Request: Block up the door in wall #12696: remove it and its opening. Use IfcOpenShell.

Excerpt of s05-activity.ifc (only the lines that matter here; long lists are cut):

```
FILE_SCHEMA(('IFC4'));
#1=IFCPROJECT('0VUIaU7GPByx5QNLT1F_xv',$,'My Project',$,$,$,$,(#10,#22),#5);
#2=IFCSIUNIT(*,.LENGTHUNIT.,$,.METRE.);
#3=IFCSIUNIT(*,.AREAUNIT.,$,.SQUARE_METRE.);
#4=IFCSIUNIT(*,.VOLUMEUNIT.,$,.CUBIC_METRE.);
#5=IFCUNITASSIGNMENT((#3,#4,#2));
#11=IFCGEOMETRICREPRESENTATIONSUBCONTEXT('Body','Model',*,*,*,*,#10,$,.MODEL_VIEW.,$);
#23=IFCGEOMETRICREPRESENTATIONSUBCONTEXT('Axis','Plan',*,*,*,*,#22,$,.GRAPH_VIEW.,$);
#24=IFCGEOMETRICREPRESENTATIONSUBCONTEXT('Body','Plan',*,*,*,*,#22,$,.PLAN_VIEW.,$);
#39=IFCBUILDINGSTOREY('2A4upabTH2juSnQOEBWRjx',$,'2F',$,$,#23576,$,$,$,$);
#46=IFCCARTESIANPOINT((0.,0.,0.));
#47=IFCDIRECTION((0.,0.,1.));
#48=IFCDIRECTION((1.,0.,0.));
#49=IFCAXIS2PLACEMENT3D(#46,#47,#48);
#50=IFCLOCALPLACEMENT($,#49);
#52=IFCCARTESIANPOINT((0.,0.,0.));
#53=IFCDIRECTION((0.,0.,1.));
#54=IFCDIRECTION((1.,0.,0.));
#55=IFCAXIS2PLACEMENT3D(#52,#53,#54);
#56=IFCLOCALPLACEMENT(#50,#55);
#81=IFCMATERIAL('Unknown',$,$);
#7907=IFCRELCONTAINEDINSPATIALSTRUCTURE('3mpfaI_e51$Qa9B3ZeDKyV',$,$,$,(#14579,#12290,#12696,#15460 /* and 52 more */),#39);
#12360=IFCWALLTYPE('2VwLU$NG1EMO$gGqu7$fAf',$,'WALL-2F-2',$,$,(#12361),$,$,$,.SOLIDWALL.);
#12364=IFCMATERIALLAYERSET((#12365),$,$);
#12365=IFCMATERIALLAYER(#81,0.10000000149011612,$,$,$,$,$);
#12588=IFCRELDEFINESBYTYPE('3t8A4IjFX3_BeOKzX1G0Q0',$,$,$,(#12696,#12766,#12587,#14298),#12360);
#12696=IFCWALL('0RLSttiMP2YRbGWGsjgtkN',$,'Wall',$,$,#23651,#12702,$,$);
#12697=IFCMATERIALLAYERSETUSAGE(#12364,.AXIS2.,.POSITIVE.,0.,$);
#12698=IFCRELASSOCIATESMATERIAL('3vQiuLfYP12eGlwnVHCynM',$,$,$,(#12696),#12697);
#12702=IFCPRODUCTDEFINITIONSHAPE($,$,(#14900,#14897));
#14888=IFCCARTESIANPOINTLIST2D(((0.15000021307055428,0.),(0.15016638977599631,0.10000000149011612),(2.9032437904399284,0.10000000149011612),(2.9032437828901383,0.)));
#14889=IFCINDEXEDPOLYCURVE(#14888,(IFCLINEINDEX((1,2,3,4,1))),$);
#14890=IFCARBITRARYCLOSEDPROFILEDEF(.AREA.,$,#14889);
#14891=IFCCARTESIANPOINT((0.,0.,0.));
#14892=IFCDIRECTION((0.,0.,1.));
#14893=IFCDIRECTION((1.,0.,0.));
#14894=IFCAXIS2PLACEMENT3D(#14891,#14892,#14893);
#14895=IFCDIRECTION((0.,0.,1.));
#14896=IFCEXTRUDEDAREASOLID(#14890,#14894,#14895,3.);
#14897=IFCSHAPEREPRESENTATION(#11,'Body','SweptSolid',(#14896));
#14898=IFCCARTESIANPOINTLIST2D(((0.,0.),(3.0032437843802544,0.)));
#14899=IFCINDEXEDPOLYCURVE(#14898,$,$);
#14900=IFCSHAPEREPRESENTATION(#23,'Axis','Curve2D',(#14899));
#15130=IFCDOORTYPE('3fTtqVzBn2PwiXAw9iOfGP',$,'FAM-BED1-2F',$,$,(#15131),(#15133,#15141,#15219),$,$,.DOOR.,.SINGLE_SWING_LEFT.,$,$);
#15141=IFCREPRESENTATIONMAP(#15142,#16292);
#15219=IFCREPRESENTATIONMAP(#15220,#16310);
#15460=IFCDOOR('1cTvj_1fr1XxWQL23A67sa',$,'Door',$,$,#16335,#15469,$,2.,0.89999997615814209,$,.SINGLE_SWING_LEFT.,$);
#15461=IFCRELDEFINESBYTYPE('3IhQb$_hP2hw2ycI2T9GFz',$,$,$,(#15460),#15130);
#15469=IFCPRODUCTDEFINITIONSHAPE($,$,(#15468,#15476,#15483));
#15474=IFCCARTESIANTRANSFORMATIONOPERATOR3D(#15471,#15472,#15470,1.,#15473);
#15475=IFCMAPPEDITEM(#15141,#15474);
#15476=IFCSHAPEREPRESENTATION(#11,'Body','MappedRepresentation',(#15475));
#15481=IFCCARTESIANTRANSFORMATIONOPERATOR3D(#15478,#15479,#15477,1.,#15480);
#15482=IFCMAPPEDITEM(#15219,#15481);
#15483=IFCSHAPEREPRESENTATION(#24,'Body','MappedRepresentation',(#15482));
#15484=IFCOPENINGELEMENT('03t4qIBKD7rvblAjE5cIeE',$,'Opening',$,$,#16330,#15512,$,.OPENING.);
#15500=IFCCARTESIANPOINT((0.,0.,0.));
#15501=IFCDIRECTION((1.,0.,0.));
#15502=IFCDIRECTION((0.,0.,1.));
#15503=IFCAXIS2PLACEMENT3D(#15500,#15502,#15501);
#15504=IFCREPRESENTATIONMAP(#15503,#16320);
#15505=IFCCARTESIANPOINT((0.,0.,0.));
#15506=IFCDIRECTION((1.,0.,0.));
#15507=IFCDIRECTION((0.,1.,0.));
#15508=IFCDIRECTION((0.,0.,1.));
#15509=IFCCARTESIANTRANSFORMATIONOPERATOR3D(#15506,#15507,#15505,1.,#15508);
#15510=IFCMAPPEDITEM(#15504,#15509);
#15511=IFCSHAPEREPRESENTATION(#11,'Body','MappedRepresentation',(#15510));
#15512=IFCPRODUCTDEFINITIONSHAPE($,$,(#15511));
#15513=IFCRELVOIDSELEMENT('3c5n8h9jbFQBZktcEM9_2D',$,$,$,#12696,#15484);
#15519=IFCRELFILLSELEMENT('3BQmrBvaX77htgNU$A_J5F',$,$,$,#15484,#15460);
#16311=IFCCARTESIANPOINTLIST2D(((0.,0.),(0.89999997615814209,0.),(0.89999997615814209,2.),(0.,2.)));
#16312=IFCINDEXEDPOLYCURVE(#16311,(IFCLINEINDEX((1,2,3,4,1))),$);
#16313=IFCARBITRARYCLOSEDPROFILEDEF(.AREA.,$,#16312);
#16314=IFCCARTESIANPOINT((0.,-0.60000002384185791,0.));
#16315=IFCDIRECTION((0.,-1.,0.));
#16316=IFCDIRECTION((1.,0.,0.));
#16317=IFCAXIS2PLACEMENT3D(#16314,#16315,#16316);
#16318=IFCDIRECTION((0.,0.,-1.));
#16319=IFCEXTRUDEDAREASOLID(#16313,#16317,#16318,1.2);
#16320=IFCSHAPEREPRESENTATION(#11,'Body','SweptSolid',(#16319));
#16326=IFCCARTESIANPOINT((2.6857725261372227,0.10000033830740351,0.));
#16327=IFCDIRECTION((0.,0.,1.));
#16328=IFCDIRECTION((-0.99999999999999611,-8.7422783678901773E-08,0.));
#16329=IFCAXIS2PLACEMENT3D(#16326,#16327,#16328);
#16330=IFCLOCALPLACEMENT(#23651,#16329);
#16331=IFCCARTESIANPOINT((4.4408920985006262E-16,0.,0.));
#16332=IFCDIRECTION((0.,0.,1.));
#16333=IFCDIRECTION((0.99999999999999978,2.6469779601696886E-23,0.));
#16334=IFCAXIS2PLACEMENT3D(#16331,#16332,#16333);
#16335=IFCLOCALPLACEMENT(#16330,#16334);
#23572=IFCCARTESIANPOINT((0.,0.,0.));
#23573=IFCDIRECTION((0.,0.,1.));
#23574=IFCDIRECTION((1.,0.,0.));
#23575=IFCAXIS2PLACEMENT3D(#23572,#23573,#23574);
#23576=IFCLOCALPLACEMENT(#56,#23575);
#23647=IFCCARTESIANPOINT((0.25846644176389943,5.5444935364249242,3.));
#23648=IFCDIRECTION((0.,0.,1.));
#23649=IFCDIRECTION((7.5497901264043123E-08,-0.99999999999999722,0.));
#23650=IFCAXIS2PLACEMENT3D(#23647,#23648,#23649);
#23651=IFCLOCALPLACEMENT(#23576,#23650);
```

```python
import ifcopenshell
import ifcopenshell.api.feature
import ifcopenshell.api.root
import ifcopenshell.geom
import ifcopenshell.util.shape

model = ifcopenshell.open("s05-activity.ifc")
settings = ifcopenshell.geom.settings()


def volume(element):
    """Net volume in cubic metres, openings subtracted."""
    shape = ifcopenshell.geom.create_shape(settings, element)
    return ifcopenshell.util.shape.get_volume(shape.geometry)


door = model.by_guid("1cTvj_1fr1XxWQL23A67sa")
opening = door.FillsVoids[0].RelatingOpeningElement
wall = opening.VoidsElements[0].RelatingBuildingElement
before = volume(wall)

ifcopenshell.api.root.remove_product(model, product=door)
ifcopenshell.api.feature.remove_feature(model, feature=opening)

after = volume(wall)

print(f"wall volume {before:.3f} -> {after:.3f} m3")

model.write("s05-activity_updated.ifc")
```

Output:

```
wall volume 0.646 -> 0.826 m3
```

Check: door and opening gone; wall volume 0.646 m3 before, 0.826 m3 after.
